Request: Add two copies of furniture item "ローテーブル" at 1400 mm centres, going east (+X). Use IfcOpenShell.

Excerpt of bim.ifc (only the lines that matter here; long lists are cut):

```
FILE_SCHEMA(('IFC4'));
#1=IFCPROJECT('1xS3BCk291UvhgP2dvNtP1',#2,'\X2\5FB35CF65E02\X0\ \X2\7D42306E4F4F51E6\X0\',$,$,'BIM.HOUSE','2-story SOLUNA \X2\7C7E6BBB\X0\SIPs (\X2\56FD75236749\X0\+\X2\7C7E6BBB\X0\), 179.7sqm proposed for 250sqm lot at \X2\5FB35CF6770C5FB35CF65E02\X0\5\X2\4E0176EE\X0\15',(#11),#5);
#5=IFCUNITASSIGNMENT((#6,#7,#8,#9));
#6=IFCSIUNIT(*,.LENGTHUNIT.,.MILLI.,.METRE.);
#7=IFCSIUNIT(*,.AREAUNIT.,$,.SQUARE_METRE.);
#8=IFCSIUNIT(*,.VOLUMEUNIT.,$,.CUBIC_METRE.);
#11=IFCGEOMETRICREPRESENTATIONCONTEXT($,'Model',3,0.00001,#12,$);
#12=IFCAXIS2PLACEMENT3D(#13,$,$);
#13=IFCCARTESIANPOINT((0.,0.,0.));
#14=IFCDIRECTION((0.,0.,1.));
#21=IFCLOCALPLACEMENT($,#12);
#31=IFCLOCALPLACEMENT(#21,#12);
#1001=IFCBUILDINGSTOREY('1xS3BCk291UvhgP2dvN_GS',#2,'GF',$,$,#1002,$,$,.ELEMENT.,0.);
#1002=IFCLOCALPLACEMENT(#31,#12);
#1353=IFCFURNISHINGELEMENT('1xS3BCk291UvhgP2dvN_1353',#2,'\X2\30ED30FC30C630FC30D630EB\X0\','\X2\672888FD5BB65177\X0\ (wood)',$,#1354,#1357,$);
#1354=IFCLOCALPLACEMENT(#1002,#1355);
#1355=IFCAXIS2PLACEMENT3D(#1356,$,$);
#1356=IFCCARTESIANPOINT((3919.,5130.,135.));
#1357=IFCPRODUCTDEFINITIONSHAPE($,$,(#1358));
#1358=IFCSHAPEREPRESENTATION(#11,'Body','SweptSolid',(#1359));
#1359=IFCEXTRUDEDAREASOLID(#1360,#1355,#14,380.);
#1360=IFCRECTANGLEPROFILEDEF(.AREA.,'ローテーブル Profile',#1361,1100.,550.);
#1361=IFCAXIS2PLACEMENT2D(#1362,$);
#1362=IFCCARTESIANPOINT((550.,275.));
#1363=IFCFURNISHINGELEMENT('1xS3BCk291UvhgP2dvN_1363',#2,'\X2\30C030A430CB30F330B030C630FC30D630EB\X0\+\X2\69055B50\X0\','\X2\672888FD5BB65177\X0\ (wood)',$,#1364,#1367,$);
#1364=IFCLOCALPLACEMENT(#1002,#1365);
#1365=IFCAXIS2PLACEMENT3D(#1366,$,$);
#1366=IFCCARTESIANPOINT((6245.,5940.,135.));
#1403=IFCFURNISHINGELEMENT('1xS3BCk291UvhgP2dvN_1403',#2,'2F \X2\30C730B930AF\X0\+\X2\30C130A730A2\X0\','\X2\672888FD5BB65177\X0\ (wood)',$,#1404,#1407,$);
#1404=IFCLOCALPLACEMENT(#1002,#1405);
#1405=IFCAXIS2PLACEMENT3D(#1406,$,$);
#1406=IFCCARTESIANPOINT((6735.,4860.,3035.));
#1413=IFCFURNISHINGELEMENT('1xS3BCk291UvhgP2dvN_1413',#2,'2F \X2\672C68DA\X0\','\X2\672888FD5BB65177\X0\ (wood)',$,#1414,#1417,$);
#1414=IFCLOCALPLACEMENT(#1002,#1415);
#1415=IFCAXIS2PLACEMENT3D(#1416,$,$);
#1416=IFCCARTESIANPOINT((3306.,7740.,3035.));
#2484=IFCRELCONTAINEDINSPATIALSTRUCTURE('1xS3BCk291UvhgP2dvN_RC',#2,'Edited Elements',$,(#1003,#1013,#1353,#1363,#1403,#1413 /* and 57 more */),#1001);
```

```python
import numpy as np
import ifcopenshell
import ifcopenshell.api.geometry
import ifcopenshell.api.root
import ifcopenshell.util.element
import ifcopenshell.util.placement

model = ifcopenshell.open("bim.ifc")


def reuse_history(source, copy):
    """copy_class also copies each property set's owner history, people and application; keep the originals."""
    for rel in copy.IsDefinedBy:
        if rel.is_a("IfcRelDefinesByProperties") and (history := rel.RelatingPropertyDefinition.OwnerHistory):
            rel.RelatingPropertyDefinition.OwnerHistory = source.OwnerHistory
            ifcopenshell.util.element.remove_deep2(model, history)


source = model.by_guid("1xS3BCk291UvhgP2dvN_1353")
base = ifcopenshell.util.placement.get_local_placement(source.ObjectPlacement)
step = np.array([1.0, 0.0, 0.0]) * 1400.0

for i in range(1, 3):
    copy = ifcopenshell.api.root.copy_class(model, product=source)
    copy.Representation = ifcopenshell.util.element.copy_deep(
        model, source.Representation, exclude=["IfcGeometricRepresentationContext", "IfcRepresentationMap"]
    )
    reuse_history(source, copy)
    matrix = base.copy()
    matrix[:3, 3] += i * step
    print("added at", matrix[:3, 3].round(3) + 0.0)
    ifcopenshell.api.geometry.edit_object_placement(model, product=copy, matrix=matrix, is_si=False)

model.write("bim_v2.ifc")
```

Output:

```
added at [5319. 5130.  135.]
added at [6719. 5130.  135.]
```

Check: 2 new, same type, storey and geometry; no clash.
